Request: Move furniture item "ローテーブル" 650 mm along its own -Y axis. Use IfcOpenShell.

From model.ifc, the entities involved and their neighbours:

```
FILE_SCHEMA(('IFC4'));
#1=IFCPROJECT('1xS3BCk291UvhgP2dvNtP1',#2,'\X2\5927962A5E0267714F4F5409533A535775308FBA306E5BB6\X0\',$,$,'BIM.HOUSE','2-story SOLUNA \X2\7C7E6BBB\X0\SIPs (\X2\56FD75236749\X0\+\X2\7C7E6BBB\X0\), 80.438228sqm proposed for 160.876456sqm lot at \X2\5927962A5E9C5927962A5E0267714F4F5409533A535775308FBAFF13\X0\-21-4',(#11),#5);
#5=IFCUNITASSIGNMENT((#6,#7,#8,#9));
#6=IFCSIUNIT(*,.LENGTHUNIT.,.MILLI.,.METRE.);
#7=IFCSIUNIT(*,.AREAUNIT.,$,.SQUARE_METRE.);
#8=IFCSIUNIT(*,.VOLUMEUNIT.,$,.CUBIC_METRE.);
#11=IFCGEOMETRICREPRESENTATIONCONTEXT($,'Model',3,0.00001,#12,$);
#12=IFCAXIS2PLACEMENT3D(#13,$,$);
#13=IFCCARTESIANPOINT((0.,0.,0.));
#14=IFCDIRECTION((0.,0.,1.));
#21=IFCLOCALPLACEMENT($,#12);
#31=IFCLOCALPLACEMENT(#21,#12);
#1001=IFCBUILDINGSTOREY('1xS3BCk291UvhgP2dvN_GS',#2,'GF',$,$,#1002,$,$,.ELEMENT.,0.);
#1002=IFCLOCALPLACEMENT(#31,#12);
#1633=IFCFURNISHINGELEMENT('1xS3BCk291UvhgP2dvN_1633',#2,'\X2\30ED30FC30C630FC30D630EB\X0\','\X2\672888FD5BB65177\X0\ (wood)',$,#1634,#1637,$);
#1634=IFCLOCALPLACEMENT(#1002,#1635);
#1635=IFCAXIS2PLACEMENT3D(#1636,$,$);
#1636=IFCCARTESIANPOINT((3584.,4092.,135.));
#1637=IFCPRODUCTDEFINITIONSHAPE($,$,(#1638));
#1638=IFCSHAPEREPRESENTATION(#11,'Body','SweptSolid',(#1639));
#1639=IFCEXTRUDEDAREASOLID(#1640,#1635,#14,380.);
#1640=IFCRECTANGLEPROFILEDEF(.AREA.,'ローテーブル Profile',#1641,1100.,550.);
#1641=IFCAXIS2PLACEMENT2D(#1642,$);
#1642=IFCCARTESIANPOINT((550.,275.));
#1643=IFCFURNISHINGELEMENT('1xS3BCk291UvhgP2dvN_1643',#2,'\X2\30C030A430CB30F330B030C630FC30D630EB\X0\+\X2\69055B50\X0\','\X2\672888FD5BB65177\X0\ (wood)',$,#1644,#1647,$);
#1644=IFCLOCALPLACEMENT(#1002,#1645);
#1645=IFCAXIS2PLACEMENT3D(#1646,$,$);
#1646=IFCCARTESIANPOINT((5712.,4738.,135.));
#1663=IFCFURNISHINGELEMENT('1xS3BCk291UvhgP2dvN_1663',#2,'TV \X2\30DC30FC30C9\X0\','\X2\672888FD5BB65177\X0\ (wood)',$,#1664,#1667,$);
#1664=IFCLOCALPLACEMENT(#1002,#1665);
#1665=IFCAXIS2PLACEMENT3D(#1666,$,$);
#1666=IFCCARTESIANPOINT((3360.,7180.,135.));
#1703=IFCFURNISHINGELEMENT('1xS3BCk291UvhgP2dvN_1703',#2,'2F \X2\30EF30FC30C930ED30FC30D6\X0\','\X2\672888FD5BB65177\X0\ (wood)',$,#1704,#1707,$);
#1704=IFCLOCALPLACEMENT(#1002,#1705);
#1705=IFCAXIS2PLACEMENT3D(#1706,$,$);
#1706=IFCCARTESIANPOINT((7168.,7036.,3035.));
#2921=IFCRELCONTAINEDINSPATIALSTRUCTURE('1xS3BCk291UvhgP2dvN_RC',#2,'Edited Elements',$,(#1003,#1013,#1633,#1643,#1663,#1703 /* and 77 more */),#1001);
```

```python
import ifcopenshell
import ifcopenshell.api.geometry
import ifcopenshell.util.placement
import ifcopenshell.util.unit

model = ifcopenshell.open("model.ifc")
unit_scale = ifcopenshell.util.unit.calculate_unit_scale(model)

item = model.by_guid("1xS3BCk291UvhgP2dvN_1633")
matrix = ifcopenshell.util.placement.get_local_placement(item.ObjectPlacement)
matrix[:3, 3] -= matrix[:3, 1] * 0.65 / unit_scale
ifcopenshell.api.geometry.edit_object_placement(model, product=item, matrix=matrix, is_si=False)

print(ifcopenshell.util.placement.get_local_placement(item.ObjectPlacement).round(3) + 0.0)

model.write("model_updated.ifc")
```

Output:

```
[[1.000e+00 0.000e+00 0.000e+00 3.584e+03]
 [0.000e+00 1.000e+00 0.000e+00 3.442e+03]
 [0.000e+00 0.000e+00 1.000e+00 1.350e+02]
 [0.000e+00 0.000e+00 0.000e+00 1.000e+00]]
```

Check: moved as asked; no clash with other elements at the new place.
